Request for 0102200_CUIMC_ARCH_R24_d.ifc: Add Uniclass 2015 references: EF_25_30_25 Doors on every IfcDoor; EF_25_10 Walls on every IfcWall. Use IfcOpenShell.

First a look at what the model holds.

```python
import ifcopenshell

model = ifcopenshell.open("0102200_CUIMC_ARCH_R24_d.ifc")
print(model.schema)
print("classifications:", [c.Name for c in model.by_type("IfcClassification")])
for ifc_class in ("IfcDoor", "IfcRoof", "IfcStair", "IfcWall", "IfcWindow"):
    print(ifc_class, len(model.by_type(ifc_class)))
```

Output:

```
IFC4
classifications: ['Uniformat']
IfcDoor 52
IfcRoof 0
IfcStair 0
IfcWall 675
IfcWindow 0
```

```python
import ifcopenshell
import ifcopenshell.api.classification

model = ifcopenshell.open("0102200_CUIMC_ARCH_R24_d.ifc")

system = ifcopenshell.api.classification.add_classification(model, classification="Uniclass 2015")

codes = {
    "IfcDoor": ("EF_25_30_25", "Doors"),
    "IfcWall": ("EF_25_10", "Walls"),
}
for ifc_class, (code, name) in codes.items():
    products = model.by_type(ifc_class)
    ifcopenshell.api.classification.add_reference(
        model, products=products, classification=system, identification=code, name=name
    )
    print(code, len(products))

model.write("0102200_CUIMC_ARCH_R24_d_v2.ifc")
```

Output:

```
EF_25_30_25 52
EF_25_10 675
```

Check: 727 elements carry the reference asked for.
